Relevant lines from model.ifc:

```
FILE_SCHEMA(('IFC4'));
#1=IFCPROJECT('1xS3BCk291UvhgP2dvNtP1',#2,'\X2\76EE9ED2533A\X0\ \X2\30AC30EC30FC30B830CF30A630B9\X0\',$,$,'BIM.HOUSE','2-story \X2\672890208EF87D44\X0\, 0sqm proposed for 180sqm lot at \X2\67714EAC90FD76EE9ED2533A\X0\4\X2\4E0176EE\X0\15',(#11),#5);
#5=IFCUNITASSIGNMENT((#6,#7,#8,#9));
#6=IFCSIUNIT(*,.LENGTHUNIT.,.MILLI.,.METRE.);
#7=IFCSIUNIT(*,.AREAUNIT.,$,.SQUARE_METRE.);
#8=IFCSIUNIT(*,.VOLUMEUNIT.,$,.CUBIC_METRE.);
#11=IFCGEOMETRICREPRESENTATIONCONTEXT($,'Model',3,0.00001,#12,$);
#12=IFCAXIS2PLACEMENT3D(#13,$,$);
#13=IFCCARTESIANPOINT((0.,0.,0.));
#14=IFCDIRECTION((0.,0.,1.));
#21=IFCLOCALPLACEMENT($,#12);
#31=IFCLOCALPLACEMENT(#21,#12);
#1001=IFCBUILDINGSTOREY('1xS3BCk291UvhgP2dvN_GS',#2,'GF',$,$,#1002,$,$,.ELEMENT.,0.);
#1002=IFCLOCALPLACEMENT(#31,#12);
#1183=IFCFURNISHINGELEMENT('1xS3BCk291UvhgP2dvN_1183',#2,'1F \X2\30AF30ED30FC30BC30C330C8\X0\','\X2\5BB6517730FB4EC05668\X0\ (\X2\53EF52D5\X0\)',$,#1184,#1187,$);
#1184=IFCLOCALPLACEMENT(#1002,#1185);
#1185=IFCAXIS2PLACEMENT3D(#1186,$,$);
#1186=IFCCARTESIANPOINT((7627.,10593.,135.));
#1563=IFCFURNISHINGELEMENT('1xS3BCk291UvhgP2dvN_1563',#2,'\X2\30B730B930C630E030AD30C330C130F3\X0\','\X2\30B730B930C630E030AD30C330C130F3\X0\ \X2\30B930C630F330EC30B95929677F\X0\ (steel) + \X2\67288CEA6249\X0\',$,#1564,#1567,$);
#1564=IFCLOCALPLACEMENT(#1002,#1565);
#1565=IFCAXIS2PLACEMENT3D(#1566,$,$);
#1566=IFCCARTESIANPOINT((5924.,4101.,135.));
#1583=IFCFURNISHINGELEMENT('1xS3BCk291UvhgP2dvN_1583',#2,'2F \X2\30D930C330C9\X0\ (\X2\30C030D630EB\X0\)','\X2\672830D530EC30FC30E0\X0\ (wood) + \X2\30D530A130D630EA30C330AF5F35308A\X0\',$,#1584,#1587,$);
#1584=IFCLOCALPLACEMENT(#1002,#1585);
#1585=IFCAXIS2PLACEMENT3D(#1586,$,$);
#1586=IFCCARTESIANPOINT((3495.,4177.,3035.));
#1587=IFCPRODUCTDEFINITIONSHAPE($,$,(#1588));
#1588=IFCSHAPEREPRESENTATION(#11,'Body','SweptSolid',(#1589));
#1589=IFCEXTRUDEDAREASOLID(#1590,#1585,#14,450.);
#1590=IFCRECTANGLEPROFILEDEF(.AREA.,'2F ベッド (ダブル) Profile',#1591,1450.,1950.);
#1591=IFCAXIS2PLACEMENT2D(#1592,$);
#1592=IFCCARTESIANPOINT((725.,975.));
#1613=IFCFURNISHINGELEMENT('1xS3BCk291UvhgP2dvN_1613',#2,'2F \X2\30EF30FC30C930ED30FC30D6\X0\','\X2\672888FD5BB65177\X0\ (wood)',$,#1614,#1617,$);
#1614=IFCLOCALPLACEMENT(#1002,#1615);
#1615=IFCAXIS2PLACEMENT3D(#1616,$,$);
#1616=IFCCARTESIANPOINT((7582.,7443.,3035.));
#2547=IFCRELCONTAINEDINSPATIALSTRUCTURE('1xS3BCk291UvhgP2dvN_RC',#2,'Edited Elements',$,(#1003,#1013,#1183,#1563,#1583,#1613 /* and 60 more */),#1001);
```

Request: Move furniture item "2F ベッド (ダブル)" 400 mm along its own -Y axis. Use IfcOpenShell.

```python
import ifcopenshell
import ifcopenshell.api.geometry
import ifcopenshell.util.placement
import ifcopenshell.util.unit

model = ifcopenshell.open("model.ifc")
unit_scale = ifcopenshell.util.unit.calculate_unit_scale(model)

item = model.by_id(1583)
matrix = ifcopenshell.util.placement.get_local_placement(item.ObjectPlacement)
matrix[:3, 3] -= matrix[:3, 1] * 0.4 / unit_scale
ifcopenshell.api.geometry.edit_object_placement(model, product=item, matrix=matrix, is_si=False)

print(ifcopenshell.util.placement.get_local_placement(item.ObjectPlacement).round(3) + 0.0)

model.write("model_edited.ifc")
```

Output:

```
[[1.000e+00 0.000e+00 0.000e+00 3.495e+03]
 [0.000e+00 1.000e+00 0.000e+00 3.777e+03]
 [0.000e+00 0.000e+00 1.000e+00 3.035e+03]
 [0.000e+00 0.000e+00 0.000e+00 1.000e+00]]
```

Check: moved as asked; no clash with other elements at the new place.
